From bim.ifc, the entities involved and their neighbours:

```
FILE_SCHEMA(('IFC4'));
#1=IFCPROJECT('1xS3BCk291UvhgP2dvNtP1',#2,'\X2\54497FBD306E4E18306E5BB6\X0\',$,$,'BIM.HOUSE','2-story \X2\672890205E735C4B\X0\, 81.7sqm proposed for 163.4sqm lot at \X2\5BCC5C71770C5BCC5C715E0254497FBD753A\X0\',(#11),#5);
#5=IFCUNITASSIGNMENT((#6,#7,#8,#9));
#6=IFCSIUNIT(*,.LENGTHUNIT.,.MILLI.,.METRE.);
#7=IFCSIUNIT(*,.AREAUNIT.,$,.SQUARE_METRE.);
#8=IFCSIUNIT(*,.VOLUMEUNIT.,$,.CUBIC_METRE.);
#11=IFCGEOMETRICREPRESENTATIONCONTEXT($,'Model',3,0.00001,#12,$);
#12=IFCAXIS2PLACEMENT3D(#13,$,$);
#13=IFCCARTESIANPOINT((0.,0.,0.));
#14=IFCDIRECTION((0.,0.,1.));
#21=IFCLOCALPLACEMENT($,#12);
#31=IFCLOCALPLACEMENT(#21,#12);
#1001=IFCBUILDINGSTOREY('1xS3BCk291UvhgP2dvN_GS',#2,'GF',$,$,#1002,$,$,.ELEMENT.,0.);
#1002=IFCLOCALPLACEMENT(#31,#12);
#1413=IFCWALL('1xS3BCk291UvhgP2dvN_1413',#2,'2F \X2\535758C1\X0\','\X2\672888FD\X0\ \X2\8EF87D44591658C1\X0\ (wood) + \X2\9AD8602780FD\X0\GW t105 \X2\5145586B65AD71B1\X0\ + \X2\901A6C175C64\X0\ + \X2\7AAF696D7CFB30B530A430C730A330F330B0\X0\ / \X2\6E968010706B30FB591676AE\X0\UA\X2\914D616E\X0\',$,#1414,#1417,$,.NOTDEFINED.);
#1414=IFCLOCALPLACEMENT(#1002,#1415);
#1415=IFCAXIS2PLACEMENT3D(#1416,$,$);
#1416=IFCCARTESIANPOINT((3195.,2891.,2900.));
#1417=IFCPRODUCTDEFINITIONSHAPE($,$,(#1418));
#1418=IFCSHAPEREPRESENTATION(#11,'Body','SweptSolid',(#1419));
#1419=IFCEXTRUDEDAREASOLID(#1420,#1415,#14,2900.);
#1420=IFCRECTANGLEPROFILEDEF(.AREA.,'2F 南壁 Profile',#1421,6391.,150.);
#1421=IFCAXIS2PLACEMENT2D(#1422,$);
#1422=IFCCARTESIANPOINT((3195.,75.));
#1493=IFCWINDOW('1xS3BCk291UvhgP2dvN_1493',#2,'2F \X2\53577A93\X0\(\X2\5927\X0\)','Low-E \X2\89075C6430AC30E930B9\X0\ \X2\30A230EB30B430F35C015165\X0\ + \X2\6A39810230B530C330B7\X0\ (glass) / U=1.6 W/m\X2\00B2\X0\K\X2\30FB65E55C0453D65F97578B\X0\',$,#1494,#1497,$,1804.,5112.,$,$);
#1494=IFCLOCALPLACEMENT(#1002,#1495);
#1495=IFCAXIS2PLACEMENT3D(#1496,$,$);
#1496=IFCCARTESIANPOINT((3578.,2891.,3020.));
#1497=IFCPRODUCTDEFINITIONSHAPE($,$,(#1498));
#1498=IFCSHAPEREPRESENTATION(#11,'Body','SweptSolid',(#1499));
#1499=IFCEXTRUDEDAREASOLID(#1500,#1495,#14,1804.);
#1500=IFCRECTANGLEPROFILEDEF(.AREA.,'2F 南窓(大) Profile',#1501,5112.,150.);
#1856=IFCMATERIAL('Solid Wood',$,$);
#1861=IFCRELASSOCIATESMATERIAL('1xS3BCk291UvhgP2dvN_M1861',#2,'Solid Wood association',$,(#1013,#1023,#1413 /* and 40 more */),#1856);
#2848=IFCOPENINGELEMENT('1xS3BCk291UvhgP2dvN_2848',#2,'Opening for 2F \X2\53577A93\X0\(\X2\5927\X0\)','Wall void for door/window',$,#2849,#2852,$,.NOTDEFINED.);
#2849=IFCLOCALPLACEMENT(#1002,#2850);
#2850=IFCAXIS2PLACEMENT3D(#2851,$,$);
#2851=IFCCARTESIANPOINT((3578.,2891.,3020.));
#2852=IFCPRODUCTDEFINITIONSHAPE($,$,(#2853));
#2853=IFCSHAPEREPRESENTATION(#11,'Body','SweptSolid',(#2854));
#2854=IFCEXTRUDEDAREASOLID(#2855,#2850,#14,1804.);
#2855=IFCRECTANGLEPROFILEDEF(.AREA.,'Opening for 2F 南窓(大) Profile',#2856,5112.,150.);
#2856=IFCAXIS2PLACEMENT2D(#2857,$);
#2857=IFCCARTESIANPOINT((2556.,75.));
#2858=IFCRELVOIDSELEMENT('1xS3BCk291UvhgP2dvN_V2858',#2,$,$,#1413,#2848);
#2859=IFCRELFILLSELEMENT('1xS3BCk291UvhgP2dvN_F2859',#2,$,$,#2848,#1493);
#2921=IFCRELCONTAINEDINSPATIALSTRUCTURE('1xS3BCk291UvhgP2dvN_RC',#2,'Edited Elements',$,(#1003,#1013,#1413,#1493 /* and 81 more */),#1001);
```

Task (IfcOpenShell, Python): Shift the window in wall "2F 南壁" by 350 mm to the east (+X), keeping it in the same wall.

```python
import ifcopenshell
import ifcopenshell.api.geometry
import ifcopenshell.util.placement

model = ifcopenshell.open("bim.ifc")

window = model.by_guid("1xS3BCk291UvhgP2dvN_1493")
opening = window.FillsVoids[0].RelatingOpeningElement
wall = opening.VoidsElements[0].RelatingBuildingElement

wall_matrix = ifcopenshell.util.placement.get_local_placement(wall.ObjectPlacement)
shift = wall_matrix[:3, 0] * 350.0
before = ifcopenshell.util.placement.get_local_placement(window.ObjectPlacement)[:3, 3].copy()

# The window is not placed relative to its opening, so move both.
for product in (opening, window):
    matrix = ifcopenshell.util.placement.get_local_placement(product.ObjectPlacement)
    matrix[:3, 3] += shift
    ifcopenshell.api.geometry.edit_object_placement(model, product=product, matrix=matrix, is_si=False)

after = ifcopenshell.util.placement.get_local_placement(window.ObjectPlacement)[:3, 3]
print("window moved by", (after - before).round(3) + 0.0)

model.write("bim-out.ifc")
```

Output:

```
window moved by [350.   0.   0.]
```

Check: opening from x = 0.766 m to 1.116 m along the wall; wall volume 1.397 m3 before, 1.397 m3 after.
